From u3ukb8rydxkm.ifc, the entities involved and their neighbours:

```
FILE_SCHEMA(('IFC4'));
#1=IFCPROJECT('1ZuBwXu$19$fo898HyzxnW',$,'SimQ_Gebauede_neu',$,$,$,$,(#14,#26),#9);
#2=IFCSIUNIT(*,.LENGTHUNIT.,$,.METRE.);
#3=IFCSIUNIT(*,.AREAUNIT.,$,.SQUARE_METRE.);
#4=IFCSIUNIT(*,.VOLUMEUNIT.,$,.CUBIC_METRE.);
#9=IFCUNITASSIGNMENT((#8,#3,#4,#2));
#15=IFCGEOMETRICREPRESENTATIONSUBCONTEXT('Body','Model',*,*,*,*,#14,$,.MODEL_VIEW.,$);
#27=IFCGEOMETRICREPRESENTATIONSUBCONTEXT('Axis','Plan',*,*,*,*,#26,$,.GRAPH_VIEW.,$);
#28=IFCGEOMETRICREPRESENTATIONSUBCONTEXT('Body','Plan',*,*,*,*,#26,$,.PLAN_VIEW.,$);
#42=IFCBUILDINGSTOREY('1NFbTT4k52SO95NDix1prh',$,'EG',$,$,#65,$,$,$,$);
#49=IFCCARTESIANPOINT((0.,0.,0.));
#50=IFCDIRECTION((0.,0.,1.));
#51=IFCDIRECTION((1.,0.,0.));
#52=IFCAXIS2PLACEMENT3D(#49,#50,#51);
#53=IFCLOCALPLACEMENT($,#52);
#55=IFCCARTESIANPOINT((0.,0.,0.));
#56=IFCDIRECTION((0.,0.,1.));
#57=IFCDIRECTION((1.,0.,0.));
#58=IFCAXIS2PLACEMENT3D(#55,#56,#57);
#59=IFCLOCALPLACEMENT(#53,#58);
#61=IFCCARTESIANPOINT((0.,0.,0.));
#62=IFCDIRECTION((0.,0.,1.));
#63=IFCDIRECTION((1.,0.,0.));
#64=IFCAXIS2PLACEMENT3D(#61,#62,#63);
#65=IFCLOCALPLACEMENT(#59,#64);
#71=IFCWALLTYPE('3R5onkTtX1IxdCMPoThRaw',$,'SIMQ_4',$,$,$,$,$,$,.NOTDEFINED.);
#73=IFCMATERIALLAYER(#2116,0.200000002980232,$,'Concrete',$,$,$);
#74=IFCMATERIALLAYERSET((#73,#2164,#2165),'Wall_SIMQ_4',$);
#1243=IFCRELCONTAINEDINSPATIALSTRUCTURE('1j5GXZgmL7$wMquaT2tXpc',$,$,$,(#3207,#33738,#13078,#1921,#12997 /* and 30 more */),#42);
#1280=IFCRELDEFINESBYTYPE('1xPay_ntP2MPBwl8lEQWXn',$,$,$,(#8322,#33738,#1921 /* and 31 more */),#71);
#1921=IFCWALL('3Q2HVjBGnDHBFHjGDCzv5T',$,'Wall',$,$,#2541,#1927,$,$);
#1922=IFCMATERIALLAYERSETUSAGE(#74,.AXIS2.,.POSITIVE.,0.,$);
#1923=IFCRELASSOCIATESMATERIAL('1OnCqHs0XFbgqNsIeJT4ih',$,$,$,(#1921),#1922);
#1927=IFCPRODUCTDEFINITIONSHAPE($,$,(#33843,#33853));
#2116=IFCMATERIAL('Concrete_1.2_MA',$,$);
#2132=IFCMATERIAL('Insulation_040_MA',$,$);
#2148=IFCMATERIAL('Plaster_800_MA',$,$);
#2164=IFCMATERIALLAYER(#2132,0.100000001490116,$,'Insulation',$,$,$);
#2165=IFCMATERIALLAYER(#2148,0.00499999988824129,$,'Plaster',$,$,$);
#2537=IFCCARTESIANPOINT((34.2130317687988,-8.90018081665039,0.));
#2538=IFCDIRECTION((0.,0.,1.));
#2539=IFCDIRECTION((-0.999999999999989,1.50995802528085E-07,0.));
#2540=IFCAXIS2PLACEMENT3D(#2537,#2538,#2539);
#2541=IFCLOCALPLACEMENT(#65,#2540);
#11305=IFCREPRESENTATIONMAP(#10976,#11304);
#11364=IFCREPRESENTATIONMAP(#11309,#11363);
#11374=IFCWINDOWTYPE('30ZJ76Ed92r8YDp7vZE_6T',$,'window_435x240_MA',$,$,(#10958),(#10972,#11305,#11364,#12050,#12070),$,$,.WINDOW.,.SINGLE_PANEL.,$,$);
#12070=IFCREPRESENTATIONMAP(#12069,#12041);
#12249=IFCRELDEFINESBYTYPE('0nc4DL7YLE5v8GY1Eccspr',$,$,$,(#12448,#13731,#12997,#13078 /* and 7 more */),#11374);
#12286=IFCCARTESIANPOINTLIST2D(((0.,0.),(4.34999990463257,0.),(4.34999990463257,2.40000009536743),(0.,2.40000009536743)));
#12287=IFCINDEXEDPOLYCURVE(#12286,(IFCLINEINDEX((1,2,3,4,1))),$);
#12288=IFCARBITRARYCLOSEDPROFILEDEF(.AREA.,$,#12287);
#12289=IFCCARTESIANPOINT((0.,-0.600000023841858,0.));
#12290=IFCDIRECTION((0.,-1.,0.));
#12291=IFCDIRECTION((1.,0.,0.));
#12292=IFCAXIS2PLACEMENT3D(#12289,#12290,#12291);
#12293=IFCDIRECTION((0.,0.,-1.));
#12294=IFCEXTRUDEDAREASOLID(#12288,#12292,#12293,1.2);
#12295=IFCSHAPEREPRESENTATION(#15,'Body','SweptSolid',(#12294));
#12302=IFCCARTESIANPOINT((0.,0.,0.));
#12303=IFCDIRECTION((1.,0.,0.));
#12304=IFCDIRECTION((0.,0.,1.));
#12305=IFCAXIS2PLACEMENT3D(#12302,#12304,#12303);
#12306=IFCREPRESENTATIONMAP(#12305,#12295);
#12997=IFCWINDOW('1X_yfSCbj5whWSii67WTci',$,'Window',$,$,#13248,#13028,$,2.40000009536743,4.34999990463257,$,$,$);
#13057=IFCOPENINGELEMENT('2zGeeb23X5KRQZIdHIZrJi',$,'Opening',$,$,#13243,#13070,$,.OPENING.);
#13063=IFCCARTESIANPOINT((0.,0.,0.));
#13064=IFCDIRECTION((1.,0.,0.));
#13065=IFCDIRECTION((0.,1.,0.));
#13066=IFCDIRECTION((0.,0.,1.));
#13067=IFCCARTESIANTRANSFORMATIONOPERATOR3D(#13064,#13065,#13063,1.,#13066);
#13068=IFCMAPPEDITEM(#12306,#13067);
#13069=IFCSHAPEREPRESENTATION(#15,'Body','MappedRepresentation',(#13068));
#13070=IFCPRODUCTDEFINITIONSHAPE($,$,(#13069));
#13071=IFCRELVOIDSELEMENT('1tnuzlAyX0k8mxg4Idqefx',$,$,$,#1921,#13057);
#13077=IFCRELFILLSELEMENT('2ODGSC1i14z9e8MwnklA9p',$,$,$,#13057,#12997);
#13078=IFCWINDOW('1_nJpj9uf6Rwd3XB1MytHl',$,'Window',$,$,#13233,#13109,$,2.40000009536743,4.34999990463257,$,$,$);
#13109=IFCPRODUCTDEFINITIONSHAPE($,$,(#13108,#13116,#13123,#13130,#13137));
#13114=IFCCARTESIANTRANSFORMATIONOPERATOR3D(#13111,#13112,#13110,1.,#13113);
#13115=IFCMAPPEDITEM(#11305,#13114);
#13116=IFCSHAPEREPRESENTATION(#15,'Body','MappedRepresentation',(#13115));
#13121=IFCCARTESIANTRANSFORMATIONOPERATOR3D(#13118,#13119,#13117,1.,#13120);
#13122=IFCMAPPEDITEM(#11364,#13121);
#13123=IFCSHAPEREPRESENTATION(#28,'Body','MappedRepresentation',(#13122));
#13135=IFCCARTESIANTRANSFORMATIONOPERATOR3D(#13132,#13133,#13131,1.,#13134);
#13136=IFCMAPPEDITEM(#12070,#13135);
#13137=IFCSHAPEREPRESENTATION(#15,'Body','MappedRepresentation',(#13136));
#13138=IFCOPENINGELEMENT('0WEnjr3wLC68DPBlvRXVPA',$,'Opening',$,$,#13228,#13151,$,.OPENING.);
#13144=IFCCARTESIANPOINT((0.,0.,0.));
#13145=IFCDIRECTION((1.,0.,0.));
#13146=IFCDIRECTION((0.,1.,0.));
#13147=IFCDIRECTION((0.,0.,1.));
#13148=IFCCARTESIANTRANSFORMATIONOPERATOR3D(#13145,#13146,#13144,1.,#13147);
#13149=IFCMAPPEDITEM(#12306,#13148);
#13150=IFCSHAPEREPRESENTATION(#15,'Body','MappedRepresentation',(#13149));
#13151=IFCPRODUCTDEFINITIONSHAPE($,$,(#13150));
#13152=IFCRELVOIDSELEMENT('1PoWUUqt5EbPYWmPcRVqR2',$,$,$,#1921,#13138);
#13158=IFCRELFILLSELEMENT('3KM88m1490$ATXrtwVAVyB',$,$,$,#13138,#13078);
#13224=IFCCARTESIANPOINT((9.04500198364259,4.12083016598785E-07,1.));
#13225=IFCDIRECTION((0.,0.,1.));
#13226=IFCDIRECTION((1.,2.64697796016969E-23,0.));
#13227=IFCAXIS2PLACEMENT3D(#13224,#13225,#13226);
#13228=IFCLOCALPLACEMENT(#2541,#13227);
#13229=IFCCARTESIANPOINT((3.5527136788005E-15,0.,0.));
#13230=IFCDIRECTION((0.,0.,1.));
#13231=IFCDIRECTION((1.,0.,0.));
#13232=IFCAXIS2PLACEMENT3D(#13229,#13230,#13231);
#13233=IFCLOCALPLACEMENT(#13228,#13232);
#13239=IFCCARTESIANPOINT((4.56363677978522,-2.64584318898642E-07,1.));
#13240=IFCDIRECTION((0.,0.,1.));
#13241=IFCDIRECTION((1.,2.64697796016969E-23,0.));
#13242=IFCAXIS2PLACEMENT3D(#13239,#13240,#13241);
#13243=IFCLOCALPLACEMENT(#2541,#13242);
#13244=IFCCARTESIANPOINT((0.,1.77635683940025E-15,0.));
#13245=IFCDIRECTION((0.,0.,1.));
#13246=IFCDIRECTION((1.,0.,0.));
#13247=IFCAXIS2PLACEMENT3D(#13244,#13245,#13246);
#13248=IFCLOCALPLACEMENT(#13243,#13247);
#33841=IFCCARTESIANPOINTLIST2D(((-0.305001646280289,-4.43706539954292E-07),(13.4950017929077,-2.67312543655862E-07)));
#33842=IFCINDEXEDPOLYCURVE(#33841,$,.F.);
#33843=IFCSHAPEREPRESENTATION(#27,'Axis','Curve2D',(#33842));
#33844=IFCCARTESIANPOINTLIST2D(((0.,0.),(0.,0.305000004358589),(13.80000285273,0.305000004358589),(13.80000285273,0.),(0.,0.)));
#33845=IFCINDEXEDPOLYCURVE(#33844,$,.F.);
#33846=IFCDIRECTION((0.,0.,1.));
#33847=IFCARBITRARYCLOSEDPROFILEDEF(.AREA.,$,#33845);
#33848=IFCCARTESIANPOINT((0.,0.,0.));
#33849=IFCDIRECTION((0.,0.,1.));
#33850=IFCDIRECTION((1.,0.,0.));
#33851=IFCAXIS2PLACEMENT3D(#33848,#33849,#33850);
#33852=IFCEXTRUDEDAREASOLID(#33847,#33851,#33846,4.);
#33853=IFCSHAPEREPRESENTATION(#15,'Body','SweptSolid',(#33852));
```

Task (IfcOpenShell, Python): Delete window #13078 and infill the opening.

```python
import ifcopenshell
import ifcopenshell.api.feature
import ifcopenshell.api.root
import ifcopenshell.geom
import ifcopenshell.util.shape

model = ifcopenshell.open("u3ukb8rydxkm.ifc")
settings = ifcopenshell.geom.settings()


def volume(element):
    """Net volume in cubic metres, openings subtracted."""
    shape = ifcopenshell.geom.create_shape(settings, element)
    return ifcopenshell.util.shape.get_volume(shape.geometry)


window = model.by_guid("1_nJpj9uf6Rwd3XB1MytHl")
opening = window.FillsVoids[0].RelatingOpeningElement
wall = opening.VoidsElements[0].RelatingBuildingElement
before = volume(wall)

ifcopenshell.api.root.remove_product(model, product=window)
ifcopenshell.api.feature.remove_feature(model, feature=opening)

after = volume(wall)

print(f"wall volume {before:.3f} -> {after:.3f} m3")

model.write("u3ukb8rydxkm-out.ifc")
```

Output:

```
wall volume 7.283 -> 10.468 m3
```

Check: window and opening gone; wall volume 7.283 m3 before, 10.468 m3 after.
